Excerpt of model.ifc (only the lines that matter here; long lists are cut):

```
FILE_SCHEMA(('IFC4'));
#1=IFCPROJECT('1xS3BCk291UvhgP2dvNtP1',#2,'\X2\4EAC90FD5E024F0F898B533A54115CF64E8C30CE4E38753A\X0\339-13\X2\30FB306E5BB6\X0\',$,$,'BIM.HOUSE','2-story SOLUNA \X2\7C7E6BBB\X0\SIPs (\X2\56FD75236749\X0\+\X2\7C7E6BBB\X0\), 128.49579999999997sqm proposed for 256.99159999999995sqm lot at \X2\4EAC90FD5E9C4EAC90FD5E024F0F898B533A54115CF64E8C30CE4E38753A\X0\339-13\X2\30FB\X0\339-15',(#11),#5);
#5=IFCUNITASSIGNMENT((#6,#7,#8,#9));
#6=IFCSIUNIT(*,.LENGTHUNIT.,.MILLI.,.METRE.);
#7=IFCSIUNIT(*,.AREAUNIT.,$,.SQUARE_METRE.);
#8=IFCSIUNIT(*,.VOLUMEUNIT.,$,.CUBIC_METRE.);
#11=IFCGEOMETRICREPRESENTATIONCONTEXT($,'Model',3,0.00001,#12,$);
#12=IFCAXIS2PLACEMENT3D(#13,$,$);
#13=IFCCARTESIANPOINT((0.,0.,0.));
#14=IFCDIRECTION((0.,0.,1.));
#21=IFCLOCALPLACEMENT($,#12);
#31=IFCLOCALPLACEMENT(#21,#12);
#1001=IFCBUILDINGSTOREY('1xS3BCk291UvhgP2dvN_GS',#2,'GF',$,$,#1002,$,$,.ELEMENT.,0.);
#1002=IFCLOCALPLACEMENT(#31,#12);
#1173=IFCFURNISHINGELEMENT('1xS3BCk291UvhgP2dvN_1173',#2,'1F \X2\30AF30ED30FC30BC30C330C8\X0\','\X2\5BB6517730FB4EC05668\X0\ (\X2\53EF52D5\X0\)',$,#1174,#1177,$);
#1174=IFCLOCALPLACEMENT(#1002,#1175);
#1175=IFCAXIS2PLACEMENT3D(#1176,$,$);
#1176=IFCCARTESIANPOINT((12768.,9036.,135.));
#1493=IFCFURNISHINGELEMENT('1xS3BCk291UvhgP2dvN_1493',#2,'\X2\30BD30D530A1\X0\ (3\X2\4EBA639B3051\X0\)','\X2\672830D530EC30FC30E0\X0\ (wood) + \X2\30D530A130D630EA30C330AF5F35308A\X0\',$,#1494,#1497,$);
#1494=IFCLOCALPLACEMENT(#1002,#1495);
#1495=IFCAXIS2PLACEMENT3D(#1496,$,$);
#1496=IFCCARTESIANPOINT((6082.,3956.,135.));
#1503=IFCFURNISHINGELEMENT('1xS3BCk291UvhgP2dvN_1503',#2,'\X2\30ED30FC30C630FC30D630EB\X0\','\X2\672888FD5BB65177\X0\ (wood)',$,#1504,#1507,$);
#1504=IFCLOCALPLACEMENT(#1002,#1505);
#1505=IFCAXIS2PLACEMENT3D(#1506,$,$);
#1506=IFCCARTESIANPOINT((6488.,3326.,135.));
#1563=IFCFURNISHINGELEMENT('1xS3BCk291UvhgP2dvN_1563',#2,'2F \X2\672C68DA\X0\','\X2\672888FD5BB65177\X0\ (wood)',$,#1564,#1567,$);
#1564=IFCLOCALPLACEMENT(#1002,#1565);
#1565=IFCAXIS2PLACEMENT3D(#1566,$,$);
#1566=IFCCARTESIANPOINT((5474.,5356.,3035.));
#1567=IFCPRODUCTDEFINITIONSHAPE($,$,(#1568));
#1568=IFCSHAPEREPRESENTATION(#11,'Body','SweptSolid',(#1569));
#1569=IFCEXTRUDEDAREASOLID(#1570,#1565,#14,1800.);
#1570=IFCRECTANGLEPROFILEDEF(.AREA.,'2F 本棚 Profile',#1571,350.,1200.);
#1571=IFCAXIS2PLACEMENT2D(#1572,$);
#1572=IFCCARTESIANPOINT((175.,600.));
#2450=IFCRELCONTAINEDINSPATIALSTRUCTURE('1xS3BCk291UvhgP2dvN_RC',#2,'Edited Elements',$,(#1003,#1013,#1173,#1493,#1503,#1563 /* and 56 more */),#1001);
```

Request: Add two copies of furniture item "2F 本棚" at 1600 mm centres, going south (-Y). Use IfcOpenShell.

```python
import numpy as np
import ifcopenshell
import ifcopenshell.api.geometry
import ifcopenshell.api.root
import ifcopenshell.util.element
import ifcopenshell.util.placement
import ifcopenshell.util.unit

model = ifcopenshell.open("model.ifc")
unit_scale = ifcopenshell.util.unit.calculate_unit_scale(model)


def reuse_history(source, copy):
    """copy_class also copies each property set's owner history, people and application; keep the originals."""
    for rel in copy.IsDefinedBy:
        if rel.is_a("IfcRelDefinesByProperties") and (history := rel.RelatingPropertyDefinition.OwnerHistory):
            rel.RelatingPropertyDefinition.OwnerHistory = source.OwnerHistory
            ifcopenshell.util.element.remove_deep2(model, history)


source = model.by_guid("1xS3BCk291UvhgP2dvN_1563")
base = ifcopenshell.util.placement.get_local_placement(source.ObjectPlacement)
step = np.array([0.0, -1.0, 0.0]) * 1.6 / unit_scale

for i in range(1, 3):
    copy = ifcopenshell.api.root.copy_class(model, product=source)
    copy.Representation = ifcopenshell.util.element.copy_deep(
        model, source.Representation, exclude=["IfcGeometricRepresentationContext", "IfcRepresentationMap"]
    )
    reuse_history(source, copy)
    matrix = base.copy()
    matrix[:3, 3] += i * step
    print("added at", matrix[:3, 3].round(3) + 0.0)
    ifcopenshell.api.geometry.edit_object_placement(model, product=copy, matrix=matrix, is_si=False)

model.write("model_v2.ifc")
```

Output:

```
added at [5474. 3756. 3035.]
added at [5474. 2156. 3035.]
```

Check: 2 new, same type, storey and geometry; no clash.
